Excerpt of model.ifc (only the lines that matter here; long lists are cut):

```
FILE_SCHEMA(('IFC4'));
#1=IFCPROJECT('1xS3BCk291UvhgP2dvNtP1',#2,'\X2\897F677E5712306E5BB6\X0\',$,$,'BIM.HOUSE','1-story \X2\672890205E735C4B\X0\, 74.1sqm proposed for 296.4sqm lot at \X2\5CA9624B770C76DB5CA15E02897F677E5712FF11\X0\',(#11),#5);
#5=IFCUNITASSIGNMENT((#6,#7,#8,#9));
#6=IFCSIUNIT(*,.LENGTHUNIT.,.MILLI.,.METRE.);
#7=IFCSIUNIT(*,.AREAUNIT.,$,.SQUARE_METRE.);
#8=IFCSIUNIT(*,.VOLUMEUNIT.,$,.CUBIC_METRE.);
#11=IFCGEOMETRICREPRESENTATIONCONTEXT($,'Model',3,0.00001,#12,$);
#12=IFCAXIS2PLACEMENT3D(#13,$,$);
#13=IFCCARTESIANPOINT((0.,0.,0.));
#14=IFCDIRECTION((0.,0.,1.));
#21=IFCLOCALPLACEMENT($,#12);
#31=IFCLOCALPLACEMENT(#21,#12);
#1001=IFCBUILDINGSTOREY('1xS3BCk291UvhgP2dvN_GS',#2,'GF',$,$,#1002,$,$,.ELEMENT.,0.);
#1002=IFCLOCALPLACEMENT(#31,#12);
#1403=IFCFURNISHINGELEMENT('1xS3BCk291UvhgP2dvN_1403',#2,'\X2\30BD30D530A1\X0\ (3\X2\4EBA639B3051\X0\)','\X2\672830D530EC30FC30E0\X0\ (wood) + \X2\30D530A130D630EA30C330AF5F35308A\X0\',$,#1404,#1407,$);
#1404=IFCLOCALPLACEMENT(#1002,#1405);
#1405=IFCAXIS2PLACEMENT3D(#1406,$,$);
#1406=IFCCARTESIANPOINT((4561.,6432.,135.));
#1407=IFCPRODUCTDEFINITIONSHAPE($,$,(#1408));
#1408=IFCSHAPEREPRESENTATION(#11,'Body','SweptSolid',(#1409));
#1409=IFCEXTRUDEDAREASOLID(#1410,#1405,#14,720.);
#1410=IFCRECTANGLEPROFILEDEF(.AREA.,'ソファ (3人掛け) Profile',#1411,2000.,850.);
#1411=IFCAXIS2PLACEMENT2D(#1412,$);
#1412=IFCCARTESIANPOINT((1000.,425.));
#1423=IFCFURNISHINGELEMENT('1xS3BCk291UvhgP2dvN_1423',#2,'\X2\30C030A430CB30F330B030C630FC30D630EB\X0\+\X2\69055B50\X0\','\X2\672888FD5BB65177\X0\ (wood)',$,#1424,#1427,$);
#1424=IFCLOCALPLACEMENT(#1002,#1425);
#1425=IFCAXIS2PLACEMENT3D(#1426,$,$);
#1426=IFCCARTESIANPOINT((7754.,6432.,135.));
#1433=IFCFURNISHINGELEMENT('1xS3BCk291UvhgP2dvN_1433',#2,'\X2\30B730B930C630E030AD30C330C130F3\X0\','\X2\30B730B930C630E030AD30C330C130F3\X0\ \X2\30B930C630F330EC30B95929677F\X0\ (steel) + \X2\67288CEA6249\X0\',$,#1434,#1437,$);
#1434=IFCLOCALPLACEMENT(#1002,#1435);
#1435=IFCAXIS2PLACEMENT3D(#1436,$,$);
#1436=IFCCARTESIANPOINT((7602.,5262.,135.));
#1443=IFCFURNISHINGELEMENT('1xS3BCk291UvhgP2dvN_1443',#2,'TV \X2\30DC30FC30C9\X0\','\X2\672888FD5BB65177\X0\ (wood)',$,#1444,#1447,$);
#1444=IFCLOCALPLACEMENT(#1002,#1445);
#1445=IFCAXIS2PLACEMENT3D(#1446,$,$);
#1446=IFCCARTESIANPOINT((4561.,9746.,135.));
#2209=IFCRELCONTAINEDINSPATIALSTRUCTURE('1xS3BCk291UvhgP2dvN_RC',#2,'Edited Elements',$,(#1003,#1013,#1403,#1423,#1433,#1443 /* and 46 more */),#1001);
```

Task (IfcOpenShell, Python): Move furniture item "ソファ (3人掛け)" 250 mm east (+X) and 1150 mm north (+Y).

```python
import ifcopenshell
import ifcopenshell.api.geometry
import ifcopenshell.util.placement

model = ifcopenshell.open("model.ifc")

item = model.by_guid("1xS3BCk291UvhgP2dvN_1403")
matrix = ifcopenshell.util.placement.get_local_placement(item.ObjectPlacement)
matrix[0, 3] += 250.0
matrix[1, 3] += 1150.0
ifcopenshell.api.geometry.edit_object_placement(model, product=item, matrix=matrix, is_si=False)

print(ifcopenshell.util.placement.get_local_placement(item.ObjectPlacement).round(3) + 0.0)

model.write("model_v2.ifc")
```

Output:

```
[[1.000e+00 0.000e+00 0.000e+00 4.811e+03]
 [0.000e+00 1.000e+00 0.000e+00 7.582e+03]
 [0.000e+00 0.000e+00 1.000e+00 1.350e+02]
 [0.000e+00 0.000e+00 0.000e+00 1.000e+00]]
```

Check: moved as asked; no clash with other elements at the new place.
